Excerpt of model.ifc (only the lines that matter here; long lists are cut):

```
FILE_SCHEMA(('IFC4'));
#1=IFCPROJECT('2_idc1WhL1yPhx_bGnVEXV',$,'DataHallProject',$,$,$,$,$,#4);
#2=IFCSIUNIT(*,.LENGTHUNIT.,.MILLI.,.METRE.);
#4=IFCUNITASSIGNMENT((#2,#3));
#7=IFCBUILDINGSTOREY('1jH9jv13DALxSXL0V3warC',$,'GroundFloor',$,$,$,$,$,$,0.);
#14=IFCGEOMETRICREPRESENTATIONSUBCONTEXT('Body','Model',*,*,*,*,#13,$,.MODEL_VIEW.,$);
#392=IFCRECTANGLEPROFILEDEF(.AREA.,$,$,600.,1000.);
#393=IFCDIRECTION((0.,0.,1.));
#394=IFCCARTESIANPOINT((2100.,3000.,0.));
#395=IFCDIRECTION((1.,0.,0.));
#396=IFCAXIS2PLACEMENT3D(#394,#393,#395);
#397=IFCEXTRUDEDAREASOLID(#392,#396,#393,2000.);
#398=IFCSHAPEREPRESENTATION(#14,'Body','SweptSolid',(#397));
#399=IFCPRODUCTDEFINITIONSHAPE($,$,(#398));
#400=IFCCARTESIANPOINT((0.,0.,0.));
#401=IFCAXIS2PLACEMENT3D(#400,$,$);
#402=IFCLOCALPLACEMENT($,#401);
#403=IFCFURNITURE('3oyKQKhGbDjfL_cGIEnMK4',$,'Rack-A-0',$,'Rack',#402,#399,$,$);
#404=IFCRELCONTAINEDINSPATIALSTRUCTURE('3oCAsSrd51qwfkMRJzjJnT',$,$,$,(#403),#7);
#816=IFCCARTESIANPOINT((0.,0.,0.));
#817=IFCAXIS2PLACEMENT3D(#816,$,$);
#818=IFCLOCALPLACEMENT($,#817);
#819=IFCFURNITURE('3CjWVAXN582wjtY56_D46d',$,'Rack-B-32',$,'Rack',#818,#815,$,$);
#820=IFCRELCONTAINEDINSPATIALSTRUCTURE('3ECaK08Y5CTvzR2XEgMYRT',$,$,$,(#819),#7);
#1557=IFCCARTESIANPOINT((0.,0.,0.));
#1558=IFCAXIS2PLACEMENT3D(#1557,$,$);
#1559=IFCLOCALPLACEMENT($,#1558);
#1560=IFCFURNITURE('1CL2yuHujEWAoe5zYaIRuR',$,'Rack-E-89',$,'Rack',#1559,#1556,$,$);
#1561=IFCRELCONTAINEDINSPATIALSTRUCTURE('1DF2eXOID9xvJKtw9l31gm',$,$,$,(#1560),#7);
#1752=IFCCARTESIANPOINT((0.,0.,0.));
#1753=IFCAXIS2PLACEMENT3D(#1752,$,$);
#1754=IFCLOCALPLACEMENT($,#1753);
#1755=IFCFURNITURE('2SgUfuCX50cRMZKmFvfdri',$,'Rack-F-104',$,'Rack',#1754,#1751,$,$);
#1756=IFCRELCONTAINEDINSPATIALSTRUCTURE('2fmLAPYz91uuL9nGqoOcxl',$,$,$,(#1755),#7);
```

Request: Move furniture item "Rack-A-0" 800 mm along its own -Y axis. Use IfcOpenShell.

```python
import ifcopenshell
import ifcopenshell.api.geometry
import ifcopenshell.util.placement
import ifcopenshell.util.unit

model = ifcopenshell.open("model.ifc")
unit_scale = ifcopenshell.util.unit.calculate_unit_scale(model)

item = model.by_guid("3oyKQKhGbDjfL_cGIEnMK4")
matrix = ifcopenshell.util.placement.get_local_placement(item.ObjectPlacement)
matrix[:3, 3] -= matrix[:3, 1] * 0.8 / unit_scale
ifcopenshell.api.geometry.edit_object_placement(model, product=item, matrix=matrix, is_si=False)

print(ifcopenshell.util.placement.get_local_placement(item.ObjectPlacement).round(3) + 0.0)

model.write("model_edited.ifc")
```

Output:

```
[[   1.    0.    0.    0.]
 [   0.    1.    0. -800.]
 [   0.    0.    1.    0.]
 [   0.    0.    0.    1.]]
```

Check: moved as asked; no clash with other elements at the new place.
